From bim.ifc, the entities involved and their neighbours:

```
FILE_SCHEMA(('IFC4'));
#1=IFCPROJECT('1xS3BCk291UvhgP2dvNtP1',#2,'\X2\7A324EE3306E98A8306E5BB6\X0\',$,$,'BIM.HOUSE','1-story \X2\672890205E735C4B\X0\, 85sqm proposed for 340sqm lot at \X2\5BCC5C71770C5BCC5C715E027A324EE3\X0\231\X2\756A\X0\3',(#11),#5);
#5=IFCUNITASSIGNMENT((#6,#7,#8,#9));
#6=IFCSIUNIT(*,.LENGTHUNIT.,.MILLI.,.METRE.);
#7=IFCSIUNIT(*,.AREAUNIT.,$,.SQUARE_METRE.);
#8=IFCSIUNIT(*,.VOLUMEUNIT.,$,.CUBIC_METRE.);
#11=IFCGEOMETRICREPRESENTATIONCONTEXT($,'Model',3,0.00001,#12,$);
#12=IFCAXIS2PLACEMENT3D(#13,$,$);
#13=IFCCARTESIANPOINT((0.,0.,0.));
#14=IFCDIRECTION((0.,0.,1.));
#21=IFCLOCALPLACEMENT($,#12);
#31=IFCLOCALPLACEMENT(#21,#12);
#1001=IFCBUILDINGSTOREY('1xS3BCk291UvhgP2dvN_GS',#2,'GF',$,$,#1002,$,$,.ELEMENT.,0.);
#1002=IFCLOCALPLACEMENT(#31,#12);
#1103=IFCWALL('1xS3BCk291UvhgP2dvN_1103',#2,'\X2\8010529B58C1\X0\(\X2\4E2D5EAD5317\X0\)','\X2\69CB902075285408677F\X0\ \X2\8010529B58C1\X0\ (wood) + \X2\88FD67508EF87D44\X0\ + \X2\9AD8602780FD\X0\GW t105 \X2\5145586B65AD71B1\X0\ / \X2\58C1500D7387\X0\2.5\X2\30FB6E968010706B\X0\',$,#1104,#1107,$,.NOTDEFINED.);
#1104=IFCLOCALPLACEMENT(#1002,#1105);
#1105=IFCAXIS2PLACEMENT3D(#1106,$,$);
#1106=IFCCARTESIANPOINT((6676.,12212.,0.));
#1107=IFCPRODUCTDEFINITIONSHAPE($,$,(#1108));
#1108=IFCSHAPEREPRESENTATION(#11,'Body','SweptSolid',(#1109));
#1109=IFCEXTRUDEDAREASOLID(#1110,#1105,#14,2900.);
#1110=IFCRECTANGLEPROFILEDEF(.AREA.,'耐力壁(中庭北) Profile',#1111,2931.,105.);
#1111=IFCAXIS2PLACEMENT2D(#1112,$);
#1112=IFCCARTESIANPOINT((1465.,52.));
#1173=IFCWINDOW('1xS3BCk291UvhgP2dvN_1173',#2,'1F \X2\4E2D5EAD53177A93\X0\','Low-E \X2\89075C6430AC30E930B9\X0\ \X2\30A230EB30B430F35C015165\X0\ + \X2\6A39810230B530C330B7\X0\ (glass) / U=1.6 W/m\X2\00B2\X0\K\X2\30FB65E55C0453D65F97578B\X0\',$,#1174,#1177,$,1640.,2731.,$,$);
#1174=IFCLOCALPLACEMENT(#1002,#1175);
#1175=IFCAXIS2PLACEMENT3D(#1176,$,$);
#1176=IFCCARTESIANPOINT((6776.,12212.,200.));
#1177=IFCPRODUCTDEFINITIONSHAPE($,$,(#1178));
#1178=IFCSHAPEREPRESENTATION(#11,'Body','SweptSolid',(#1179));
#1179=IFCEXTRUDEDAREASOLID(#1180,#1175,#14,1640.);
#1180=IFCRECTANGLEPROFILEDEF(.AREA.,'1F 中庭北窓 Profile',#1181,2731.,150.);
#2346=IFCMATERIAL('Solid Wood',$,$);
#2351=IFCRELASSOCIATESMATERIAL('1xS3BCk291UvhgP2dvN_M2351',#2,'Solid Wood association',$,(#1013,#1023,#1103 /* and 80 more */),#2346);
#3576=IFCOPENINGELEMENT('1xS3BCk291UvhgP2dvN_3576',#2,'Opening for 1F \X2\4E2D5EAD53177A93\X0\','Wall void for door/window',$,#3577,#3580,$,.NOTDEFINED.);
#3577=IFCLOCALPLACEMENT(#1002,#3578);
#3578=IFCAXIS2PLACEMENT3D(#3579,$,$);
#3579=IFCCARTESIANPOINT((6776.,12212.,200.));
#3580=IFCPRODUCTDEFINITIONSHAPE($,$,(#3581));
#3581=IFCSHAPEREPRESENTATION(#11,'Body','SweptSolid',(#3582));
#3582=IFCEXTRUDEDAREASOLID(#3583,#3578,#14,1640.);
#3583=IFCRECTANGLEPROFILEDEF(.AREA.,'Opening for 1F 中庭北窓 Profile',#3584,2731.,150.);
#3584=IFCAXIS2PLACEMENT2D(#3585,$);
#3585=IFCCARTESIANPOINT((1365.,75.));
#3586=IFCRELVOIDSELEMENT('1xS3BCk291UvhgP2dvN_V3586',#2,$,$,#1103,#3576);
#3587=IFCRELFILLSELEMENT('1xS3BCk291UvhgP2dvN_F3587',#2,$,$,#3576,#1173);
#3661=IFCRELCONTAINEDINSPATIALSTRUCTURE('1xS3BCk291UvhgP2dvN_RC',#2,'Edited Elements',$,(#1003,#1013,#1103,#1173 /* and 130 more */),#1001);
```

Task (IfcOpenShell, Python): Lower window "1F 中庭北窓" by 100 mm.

```python
import numpy as np
import ifcopenshell
import ifcopenshell.api.geometry
import ifcopenshell.util.placement
import ifcopenshell.util.unit

model = ifcopenshell.open("bim.ifc")
unit_scale = ifcopenshell.util.unit.calculate_unit_scale(model)

window = model.by_guid("1xS3BCk291UvhgP2dvN_1173")
opening = window.FillsVoids[0].RelatingOpeningElement
dz = -100.0

shift = np.array([0.0, 0.0, dz])
# The window is not placed relative to its opening, so move both.
for product in (opening, window):
    matrix = ifcopenshell.util.placement.get_local_placement(product.ObjectPlacement)
    matrix[:3, 3] += shift
    ifcopenshell.api.geometry.edit_object_placement(model, product=product, matrix=matrix, is_si=False)

print(f"moved by {dz * unit_scale:+.3f} m")

model.write("bim_edited.ifc")
```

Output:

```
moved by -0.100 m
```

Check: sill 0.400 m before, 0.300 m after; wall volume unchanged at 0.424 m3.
